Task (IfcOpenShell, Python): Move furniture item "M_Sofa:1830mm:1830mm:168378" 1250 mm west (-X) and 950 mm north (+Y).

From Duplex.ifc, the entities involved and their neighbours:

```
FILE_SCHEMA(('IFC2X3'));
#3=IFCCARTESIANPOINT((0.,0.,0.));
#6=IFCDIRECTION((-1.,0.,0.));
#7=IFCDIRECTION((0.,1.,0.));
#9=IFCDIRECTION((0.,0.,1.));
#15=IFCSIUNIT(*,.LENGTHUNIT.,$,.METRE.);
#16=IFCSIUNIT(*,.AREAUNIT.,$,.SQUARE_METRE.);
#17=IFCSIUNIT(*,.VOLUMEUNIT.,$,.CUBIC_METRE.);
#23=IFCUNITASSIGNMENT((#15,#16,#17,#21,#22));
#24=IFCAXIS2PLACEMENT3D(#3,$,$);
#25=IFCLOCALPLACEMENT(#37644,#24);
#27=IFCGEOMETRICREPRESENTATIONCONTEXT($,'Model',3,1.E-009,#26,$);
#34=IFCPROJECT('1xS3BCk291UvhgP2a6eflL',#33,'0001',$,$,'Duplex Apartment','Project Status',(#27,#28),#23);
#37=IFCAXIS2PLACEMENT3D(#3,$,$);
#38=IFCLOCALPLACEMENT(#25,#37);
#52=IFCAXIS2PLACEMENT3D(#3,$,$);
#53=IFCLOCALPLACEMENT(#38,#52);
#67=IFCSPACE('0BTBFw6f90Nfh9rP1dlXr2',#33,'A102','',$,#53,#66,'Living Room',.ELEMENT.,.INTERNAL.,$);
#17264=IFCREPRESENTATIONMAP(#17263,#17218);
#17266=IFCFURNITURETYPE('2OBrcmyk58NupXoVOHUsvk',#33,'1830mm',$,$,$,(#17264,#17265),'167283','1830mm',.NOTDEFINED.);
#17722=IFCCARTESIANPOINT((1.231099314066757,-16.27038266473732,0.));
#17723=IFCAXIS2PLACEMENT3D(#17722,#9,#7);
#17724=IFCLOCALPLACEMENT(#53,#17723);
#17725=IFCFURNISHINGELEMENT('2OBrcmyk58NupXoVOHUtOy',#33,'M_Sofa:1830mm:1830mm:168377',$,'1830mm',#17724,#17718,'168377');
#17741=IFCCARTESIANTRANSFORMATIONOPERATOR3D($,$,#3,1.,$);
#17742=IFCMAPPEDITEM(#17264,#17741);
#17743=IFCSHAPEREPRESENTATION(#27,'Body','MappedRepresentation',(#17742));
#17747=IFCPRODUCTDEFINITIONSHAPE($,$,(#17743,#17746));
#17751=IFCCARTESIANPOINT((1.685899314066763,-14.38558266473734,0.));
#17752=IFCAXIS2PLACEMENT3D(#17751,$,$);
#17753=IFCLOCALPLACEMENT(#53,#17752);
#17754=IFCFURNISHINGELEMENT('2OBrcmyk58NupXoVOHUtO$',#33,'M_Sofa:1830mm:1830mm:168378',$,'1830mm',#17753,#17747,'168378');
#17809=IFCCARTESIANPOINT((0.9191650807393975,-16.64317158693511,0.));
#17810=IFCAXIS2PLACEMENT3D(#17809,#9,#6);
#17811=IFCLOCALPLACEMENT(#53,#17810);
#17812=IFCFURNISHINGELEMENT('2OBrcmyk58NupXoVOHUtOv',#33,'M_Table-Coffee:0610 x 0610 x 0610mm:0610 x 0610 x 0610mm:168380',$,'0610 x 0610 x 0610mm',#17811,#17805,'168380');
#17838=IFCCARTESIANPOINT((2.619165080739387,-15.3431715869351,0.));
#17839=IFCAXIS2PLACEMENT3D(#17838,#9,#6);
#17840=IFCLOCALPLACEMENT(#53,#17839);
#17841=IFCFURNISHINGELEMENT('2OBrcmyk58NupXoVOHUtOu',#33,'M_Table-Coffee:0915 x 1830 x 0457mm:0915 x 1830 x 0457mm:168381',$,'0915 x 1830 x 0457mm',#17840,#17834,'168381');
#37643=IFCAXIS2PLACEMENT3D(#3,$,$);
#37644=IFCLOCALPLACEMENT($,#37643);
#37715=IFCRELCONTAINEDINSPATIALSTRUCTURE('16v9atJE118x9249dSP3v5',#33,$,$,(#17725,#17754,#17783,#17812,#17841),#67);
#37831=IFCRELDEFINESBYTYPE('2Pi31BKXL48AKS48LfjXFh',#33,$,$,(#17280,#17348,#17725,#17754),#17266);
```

```python
import ifcopenshell
import ifcopenshell.api.geometry
import ifcopenshell.util.placement
import ifcopenshell.util.unit

model = ifcopenshell.open("Duplex.ifc")
unit_scale = ifcopenshell.util.unit.calculate_unit_scale(model)

item = model.by_id(17754)
matrix = ifcopenshell.util.placement.get_local_placement(item.ObjectPlacement)
matrix[0, 3] -= 1.25 / unit_scale
matrix[1, 3] += 0.95 / unit_scale
ifcopenshell.api.geometry.edit_object_placement(model, product=item, matrix=matrix, is_si=False)

print(ifcopenshell.util.placement.get_local_placement(item.ObjectPlacement).round(3) + 0.0)

model.write("Duplex_rev.ifc")
```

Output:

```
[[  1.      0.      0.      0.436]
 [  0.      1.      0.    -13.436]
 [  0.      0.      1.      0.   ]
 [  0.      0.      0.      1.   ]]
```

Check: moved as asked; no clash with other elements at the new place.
